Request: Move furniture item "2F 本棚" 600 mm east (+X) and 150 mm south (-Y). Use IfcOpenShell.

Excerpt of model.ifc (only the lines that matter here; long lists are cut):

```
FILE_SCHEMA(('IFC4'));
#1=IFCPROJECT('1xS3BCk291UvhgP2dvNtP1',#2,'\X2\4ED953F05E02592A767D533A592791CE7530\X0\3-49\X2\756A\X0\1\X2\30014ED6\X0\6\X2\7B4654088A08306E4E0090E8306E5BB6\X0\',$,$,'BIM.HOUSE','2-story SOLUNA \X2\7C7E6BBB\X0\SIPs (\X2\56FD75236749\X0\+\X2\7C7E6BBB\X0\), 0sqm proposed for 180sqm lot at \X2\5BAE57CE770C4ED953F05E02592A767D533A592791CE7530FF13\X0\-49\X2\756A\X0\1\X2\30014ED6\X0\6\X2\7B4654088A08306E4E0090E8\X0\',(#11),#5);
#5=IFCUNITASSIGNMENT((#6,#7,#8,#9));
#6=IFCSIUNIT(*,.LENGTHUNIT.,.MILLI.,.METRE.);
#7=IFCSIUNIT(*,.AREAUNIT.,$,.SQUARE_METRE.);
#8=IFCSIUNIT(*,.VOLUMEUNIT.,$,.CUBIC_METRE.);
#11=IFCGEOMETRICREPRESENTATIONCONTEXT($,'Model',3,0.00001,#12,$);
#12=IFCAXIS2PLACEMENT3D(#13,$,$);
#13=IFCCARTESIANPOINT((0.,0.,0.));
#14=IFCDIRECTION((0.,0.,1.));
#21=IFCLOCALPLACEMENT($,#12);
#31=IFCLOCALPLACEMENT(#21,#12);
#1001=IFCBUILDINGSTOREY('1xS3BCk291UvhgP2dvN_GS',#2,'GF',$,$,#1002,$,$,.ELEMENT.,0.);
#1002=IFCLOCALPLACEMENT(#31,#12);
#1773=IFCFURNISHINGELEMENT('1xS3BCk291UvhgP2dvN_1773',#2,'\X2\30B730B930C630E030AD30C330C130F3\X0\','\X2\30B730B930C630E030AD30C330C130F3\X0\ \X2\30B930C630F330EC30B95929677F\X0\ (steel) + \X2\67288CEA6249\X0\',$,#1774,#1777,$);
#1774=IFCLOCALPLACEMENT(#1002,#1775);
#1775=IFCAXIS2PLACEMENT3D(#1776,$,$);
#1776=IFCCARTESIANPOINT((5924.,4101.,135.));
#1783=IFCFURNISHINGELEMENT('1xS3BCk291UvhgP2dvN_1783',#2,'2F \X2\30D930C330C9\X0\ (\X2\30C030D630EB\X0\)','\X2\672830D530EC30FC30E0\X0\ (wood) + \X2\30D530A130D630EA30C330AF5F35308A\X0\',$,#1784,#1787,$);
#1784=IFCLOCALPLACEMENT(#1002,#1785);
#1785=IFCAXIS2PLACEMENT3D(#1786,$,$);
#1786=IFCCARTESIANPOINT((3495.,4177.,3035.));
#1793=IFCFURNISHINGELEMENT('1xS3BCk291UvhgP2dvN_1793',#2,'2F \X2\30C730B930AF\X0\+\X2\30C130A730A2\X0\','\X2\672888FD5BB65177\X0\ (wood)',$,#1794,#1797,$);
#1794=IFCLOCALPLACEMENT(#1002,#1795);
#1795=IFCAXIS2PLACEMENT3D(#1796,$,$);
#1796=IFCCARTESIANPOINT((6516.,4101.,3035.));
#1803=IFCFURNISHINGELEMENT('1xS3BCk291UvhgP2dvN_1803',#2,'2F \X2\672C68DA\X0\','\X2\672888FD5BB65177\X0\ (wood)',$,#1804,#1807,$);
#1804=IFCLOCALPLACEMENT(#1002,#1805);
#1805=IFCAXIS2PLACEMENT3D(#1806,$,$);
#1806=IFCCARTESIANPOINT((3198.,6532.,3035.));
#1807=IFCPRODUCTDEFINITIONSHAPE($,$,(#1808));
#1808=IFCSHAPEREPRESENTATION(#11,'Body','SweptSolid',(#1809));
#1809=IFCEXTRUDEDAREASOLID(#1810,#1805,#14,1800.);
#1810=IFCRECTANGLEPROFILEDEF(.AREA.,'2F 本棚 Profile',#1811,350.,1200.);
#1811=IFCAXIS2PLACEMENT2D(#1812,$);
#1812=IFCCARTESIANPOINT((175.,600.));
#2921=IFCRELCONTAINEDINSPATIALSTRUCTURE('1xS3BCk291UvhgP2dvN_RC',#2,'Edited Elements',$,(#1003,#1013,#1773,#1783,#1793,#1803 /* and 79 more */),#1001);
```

```python
import ifcopenshell
import ifcopenshell.api.geometry
import ifcopenshell.util.placement
import ifcopenshell.util.unit

model = ifcopenshell.open("model.ifc")
unit_scale = ifcopenshell.util.unit.calculate_unit_scale(model)

item = model.by_guid("1xS3BCk291UvhgP2dvN_1803")
matrix = ifcopenshell.util.placement.get_local_placement(item.ObjectPlacement)
matrix[0, 3] += 0.6 / unit_scale
matrix[1, 3] -= 0.15 / unit_scale
ifcopenshell.api.geometry.edit_object_placement(model, product=item, matrix=matrix, is_si=False)

print(ifcopenshell.util.placement.get_local_placement(item.ObjectPlacement).round(3) + 0.0)

model.write("model_updated.ifc")
```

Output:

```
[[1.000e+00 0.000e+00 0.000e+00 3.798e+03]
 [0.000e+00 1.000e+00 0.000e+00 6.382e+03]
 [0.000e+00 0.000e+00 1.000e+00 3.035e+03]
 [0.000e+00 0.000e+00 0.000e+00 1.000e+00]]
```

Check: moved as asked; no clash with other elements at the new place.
